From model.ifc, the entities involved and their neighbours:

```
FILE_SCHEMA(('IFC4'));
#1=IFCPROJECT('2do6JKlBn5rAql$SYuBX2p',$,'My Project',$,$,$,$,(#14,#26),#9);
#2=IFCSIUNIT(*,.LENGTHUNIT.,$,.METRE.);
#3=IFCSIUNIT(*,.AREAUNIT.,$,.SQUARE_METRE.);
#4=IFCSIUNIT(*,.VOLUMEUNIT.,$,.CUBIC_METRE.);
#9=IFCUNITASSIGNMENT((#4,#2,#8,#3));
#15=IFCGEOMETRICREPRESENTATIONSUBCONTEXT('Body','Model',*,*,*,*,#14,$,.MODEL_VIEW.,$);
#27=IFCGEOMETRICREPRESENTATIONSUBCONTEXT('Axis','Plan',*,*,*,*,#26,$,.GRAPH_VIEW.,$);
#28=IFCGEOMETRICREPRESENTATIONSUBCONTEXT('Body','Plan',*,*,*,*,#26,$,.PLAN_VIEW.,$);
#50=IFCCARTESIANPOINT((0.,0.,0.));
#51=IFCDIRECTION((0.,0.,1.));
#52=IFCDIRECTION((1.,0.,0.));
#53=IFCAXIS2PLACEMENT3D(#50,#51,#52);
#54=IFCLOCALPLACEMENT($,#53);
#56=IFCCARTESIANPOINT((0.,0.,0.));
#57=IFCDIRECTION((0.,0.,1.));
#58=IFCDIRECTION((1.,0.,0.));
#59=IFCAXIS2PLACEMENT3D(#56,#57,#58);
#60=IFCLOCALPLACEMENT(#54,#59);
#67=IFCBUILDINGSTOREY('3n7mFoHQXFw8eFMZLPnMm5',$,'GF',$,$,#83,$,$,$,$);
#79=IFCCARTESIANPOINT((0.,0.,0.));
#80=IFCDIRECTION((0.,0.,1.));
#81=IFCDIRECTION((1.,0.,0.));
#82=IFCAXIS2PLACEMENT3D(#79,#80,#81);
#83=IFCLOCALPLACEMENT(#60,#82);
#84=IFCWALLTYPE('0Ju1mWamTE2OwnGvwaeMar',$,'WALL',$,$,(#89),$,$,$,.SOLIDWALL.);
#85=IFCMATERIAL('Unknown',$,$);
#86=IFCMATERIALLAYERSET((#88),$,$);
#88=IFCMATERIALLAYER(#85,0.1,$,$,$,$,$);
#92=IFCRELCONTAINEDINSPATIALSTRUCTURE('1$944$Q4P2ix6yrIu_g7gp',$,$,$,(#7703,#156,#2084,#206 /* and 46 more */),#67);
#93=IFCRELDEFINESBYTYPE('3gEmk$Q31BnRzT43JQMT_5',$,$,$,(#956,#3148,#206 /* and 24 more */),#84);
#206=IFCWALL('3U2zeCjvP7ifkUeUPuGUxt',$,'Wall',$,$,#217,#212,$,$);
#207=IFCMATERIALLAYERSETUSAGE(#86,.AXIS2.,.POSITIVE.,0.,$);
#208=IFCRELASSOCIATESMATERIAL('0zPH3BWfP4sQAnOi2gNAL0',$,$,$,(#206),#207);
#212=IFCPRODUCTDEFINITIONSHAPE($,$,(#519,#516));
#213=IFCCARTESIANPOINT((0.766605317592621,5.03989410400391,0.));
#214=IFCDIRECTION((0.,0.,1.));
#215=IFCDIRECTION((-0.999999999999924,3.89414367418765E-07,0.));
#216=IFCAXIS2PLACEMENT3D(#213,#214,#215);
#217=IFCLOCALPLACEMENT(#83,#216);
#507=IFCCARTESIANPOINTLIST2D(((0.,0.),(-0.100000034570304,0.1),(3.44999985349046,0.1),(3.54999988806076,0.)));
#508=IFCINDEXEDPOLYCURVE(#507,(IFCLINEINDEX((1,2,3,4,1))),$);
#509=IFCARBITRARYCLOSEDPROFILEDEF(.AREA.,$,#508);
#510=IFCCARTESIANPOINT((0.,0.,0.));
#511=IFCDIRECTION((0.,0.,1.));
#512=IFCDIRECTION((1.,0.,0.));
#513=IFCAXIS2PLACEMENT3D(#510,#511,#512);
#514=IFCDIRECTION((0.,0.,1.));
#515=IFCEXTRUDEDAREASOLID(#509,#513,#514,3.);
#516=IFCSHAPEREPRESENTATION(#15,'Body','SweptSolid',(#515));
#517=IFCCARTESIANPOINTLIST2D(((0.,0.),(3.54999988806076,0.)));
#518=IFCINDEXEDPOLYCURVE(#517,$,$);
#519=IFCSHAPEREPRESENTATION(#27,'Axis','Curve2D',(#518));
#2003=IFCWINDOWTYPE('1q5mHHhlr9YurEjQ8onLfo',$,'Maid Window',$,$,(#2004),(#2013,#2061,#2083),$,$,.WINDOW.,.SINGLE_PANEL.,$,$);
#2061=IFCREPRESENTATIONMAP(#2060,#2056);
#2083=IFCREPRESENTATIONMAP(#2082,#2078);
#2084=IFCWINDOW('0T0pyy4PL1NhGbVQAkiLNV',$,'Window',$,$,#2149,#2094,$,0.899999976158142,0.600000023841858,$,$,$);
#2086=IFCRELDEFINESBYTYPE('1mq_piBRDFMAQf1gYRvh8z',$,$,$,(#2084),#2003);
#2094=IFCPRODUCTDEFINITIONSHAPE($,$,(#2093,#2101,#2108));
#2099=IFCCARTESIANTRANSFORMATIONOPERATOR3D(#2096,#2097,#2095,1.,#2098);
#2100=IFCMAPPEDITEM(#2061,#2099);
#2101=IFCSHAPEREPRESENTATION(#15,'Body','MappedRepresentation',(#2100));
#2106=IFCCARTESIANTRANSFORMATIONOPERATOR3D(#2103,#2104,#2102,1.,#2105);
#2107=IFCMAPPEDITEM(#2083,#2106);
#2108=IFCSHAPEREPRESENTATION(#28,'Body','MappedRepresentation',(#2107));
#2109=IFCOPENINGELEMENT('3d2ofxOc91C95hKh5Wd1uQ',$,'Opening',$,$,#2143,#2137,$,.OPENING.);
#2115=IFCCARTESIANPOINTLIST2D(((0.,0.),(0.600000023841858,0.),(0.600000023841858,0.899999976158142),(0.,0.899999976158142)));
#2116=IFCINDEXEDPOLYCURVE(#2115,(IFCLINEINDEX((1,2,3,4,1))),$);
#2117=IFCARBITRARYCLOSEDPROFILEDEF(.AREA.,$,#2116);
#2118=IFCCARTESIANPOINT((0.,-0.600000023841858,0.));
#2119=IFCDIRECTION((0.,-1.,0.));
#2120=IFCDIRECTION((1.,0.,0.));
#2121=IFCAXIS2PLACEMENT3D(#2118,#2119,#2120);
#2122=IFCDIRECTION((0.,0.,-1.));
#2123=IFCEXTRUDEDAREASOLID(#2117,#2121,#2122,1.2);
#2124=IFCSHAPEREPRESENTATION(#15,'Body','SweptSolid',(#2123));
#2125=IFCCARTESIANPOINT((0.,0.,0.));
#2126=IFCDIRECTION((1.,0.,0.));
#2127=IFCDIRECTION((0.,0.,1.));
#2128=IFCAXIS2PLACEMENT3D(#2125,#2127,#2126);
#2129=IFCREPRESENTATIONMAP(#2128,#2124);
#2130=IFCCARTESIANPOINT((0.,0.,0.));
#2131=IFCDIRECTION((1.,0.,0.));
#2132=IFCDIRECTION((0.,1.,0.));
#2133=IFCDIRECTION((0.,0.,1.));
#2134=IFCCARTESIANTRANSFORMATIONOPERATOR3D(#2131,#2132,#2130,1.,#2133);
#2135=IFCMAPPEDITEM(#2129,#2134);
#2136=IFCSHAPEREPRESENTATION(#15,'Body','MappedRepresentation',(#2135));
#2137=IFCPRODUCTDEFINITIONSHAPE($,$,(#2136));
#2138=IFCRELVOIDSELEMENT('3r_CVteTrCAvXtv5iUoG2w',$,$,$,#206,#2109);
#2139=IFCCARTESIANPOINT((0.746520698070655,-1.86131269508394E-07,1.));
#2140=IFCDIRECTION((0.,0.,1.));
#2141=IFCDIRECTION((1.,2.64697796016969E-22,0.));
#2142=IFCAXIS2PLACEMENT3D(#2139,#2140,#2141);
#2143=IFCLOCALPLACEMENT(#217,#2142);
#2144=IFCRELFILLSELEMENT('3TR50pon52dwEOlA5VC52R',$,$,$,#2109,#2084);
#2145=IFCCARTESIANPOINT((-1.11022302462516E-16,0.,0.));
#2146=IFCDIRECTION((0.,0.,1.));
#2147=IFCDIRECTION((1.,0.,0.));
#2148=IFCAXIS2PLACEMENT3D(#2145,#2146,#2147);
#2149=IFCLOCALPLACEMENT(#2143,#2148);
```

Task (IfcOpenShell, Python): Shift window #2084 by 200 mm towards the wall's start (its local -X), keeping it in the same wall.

```python
import ifcopenshell
import ifcopenshell.api.geometry
import ifcopenshell.util.placement

model = ifcopenshell.open("model.ifc")

window = model.by_id(2084)
opening = window.FillsVoids[0].RelatingOpeningElement
wall = opening.VoidsElements[0].RelatingBuildingElement

wall_matrix = ifcopenshell.util.placement.get_local_placement(wall.ObjectPlacement)
shift = wall_matrix[:3, 0] * -0.2
before = ifcopenshell.util.placement.get_local_placement(window.ObjectPlacement)[:3, 3].copy()

# The window is placed relative to its opening, so it follows when the opening moves.
matrix = ifcopenshell.util.placement.get_local_placement(opening.ObjectPlacement)
matrix[:3, 3] += shift
ifcopenshell.api.geometry.edit_object_placement(
    model, product=opening, matrix=matrix, is_si=False, should_transform_children=True
)

after = ifcopenshell.util.placement.get_local_placement(window.ObjectPlacement)[:3, 3]
print("window moved by", (after - before).round(3) + 0.0)

model.write("model_edited.ifc")
```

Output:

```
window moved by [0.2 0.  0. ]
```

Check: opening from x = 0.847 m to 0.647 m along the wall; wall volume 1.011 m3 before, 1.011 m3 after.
